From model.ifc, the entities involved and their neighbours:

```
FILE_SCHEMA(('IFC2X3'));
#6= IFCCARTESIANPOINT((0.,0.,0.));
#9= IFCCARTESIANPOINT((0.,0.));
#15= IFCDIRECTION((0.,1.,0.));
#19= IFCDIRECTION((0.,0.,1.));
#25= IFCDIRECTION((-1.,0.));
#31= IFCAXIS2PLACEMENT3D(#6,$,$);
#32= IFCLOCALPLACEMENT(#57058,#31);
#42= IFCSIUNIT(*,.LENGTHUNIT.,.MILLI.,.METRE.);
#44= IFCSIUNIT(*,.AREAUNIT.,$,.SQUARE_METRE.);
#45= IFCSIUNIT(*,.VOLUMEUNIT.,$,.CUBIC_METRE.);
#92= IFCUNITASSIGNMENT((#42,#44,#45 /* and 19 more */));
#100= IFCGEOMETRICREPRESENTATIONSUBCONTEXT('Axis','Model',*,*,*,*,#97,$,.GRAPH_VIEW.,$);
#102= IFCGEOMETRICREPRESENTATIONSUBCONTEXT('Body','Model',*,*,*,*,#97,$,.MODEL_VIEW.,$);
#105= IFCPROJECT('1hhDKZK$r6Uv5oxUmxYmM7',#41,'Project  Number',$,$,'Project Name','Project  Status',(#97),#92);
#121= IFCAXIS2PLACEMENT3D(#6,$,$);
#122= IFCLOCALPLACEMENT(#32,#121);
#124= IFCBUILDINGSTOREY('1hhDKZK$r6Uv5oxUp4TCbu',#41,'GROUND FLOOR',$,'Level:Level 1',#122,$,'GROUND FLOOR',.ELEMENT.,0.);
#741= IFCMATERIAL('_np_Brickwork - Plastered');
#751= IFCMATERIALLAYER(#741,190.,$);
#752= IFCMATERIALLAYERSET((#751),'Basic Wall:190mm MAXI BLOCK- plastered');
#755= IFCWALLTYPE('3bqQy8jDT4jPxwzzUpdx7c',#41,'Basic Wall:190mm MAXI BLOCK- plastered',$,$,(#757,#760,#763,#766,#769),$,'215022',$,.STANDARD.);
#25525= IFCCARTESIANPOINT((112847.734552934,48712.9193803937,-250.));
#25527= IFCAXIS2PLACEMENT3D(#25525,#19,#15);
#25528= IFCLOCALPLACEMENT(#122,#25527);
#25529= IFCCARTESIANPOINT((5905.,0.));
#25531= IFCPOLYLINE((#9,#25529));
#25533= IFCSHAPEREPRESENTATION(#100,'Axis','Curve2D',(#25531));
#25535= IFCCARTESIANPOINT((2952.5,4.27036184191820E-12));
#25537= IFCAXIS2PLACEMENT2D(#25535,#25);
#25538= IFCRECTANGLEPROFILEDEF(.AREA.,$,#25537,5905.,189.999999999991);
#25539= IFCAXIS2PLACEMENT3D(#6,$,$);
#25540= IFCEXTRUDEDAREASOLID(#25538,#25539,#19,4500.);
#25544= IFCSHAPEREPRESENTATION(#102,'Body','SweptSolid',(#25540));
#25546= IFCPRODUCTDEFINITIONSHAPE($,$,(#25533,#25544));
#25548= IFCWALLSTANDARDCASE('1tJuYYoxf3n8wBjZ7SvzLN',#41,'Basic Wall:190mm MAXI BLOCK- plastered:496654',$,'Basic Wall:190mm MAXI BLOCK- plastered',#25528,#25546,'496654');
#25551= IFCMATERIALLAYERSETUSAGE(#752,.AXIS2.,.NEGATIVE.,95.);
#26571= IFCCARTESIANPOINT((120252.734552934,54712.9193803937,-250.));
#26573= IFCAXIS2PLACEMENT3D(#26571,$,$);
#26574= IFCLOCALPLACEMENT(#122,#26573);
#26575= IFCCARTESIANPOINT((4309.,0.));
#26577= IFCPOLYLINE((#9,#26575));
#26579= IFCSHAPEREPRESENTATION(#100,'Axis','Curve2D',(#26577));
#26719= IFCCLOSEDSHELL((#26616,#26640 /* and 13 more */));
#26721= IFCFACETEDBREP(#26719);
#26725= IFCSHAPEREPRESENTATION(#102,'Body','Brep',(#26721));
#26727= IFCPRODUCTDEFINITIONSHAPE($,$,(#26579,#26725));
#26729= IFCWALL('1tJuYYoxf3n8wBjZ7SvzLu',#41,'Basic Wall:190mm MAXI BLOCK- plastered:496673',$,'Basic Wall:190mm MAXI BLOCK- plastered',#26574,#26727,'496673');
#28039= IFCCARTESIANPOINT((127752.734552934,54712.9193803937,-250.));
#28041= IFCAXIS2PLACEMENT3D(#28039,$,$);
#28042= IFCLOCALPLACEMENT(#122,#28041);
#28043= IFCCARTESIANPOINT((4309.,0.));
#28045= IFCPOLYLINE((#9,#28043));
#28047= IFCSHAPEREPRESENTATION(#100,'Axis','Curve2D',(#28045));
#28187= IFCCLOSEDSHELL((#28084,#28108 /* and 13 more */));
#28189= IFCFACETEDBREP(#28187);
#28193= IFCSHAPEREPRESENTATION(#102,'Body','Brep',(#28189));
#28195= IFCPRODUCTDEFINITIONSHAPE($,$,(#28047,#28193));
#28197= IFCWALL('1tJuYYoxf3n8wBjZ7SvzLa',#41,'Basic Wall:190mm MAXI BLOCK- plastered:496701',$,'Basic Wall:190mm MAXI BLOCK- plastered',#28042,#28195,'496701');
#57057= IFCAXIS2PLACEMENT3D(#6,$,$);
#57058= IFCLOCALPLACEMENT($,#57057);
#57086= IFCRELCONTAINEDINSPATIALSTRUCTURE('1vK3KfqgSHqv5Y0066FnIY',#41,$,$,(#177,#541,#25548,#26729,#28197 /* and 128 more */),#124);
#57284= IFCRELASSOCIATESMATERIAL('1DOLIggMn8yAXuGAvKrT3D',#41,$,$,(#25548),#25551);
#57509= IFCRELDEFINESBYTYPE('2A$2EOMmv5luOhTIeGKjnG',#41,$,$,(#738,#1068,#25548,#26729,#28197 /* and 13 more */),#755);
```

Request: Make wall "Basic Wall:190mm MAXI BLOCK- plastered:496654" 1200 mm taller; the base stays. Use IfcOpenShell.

```python
import ifcopenshell
import ifcopenshell.geom
import ifcopenshell.util.representation
import ifcopenshell.util.shape
import ifcopenshell.util.unit

model = ifcopenshell.open("model.ifc")
unit_scale = ifcopenshell.util.unit.calculate_unit_scale(model)
settings = ifcopenshell.geom.settings()


def volume(element):
    """Net volume in cubic metres, openings subtracted."""
    shape = ifcopenshell.geom.create_shape(settings, element)
    return ifcopenshell.util.shape.get_volume(shape.geometry)


wall = model.by_guid("1tJuYYoxf3n8wBjZ7SvzLN")
before = volume(wall)

body = ifcopenshell.util.representation.get_representation(wall, "Model", "Body")
solid = body.Items[0]
old_height = solid.Depth
solid.Depth += 1.2 / unit_scale
after = volume(wall)

print(f"height {old_height:g} -> {solid.Depth:g}, volume {before:.3f} -> {after:.3f} m3")

model.write("model-out.ifc")
```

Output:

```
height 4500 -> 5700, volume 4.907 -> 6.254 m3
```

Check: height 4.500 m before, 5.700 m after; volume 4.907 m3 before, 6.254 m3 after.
